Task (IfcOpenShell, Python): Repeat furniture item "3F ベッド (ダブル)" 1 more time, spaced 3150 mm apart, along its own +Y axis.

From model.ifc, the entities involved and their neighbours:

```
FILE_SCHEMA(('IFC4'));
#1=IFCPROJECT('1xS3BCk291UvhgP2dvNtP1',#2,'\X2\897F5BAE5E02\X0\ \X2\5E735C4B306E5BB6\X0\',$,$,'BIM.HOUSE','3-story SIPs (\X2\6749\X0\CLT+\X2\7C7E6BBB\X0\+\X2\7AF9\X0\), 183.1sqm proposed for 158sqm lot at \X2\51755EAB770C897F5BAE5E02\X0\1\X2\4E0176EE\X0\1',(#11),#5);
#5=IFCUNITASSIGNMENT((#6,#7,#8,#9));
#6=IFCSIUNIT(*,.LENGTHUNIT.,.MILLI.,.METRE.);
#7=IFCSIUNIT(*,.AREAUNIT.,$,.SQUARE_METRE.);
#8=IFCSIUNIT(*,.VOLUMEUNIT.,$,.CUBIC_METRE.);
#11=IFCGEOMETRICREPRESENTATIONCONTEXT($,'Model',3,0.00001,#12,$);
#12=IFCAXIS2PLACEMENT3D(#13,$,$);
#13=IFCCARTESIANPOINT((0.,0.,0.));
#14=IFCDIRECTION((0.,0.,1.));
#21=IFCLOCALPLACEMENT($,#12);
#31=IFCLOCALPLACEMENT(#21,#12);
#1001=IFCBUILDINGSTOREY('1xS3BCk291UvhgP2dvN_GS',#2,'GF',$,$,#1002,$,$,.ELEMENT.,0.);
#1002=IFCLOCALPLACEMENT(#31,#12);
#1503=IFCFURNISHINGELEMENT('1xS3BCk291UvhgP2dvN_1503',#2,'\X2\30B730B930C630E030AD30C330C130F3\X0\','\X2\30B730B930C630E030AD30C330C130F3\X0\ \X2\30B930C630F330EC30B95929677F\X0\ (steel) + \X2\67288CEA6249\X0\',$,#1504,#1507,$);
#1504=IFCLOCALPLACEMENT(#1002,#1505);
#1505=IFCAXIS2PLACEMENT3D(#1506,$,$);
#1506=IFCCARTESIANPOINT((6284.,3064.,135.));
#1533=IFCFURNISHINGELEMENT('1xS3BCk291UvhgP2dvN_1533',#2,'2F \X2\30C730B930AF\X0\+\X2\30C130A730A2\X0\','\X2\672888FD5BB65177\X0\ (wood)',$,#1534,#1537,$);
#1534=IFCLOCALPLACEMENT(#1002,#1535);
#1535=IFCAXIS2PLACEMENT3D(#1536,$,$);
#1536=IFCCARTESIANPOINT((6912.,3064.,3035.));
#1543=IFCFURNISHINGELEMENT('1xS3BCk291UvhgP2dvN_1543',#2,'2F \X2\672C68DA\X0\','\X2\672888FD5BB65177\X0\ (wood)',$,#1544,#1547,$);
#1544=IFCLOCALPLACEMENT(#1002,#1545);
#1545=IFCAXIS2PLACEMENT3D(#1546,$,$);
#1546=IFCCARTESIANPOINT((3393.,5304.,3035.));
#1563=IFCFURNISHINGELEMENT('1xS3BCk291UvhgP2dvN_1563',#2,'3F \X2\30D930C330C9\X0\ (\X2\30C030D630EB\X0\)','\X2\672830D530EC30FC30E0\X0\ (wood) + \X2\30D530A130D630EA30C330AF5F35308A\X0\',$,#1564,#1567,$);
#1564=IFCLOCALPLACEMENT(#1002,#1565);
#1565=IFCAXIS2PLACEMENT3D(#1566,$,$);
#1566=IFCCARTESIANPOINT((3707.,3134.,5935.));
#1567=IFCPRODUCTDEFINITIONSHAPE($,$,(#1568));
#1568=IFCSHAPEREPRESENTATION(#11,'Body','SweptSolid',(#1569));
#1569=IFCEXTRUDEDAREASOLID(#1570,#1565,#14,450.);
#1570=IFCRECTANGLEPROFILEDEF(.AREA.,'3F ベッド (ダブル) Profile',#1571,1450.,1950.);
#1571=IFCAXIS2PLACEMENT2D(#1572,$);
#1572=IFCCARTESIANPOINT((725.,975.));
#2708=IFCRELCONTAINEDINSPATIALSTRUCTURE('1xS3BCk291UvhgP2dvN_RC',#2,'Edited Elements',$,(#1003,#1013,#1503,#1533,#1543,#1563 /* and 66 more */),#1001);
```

```python
import ifcopenshell
import ifcopenshell.api.geometry
import ifcopenshell.api.root
import ifcopenshell.util.element
import ifcopenshell.util.placement
import ifcopenshell.util.unit

model = ifcopenshell.open("model.ifc")
unit_scale = ifcopenshell.util.unit.calculate_unit_scale(model)


def reuse_history(source, copy):
    """copy_class also copies each property set's owner history, people and application; keep the originals."""
    for rel in copy.IsDefinedBy:
        if rel.is_a("IfcRelDefinesByProperties") and (history := rel.RelatingPropertyDefinition.OwnerHistory):
            rel.RelatingPropertyDefinition.OwnerHistory = source.OwnerHistory
            ifcopenshell.util.element.remove_deep2(model, history)


source = model.by_guid("1xS3BCk291UvhgP2dvN_1563")
base = ifcopenshell.util.placement.get_local_placement(source.ObjectPlacement)
step = base[:3, 1] * 3.15 / unit_scale

for i in range(1, 2):
    copy = ifcopenshell.api.root.copy_class(model, product=source)
    copy.Representation = ifcopenshell.util.element.copy_deep(
        model, source.Representation, exclude=["IfcGeometricRepresentationContext", "IfcRepresentationMap"]
    )
    reuse_history(source, copy)
    matrix = base.copy()
    matrix[:3, 3] += i * step
    print("added at", matrix[:3, 3].round(3) + 0.0)
    ifcopenshell.api.geometry.edit_object_placement(model, product=copy, matrix=matrix, is_si=False)

model.write("model_edited.ifc")
```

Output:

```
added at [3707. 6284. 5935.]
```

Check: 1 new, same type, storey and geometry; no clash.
